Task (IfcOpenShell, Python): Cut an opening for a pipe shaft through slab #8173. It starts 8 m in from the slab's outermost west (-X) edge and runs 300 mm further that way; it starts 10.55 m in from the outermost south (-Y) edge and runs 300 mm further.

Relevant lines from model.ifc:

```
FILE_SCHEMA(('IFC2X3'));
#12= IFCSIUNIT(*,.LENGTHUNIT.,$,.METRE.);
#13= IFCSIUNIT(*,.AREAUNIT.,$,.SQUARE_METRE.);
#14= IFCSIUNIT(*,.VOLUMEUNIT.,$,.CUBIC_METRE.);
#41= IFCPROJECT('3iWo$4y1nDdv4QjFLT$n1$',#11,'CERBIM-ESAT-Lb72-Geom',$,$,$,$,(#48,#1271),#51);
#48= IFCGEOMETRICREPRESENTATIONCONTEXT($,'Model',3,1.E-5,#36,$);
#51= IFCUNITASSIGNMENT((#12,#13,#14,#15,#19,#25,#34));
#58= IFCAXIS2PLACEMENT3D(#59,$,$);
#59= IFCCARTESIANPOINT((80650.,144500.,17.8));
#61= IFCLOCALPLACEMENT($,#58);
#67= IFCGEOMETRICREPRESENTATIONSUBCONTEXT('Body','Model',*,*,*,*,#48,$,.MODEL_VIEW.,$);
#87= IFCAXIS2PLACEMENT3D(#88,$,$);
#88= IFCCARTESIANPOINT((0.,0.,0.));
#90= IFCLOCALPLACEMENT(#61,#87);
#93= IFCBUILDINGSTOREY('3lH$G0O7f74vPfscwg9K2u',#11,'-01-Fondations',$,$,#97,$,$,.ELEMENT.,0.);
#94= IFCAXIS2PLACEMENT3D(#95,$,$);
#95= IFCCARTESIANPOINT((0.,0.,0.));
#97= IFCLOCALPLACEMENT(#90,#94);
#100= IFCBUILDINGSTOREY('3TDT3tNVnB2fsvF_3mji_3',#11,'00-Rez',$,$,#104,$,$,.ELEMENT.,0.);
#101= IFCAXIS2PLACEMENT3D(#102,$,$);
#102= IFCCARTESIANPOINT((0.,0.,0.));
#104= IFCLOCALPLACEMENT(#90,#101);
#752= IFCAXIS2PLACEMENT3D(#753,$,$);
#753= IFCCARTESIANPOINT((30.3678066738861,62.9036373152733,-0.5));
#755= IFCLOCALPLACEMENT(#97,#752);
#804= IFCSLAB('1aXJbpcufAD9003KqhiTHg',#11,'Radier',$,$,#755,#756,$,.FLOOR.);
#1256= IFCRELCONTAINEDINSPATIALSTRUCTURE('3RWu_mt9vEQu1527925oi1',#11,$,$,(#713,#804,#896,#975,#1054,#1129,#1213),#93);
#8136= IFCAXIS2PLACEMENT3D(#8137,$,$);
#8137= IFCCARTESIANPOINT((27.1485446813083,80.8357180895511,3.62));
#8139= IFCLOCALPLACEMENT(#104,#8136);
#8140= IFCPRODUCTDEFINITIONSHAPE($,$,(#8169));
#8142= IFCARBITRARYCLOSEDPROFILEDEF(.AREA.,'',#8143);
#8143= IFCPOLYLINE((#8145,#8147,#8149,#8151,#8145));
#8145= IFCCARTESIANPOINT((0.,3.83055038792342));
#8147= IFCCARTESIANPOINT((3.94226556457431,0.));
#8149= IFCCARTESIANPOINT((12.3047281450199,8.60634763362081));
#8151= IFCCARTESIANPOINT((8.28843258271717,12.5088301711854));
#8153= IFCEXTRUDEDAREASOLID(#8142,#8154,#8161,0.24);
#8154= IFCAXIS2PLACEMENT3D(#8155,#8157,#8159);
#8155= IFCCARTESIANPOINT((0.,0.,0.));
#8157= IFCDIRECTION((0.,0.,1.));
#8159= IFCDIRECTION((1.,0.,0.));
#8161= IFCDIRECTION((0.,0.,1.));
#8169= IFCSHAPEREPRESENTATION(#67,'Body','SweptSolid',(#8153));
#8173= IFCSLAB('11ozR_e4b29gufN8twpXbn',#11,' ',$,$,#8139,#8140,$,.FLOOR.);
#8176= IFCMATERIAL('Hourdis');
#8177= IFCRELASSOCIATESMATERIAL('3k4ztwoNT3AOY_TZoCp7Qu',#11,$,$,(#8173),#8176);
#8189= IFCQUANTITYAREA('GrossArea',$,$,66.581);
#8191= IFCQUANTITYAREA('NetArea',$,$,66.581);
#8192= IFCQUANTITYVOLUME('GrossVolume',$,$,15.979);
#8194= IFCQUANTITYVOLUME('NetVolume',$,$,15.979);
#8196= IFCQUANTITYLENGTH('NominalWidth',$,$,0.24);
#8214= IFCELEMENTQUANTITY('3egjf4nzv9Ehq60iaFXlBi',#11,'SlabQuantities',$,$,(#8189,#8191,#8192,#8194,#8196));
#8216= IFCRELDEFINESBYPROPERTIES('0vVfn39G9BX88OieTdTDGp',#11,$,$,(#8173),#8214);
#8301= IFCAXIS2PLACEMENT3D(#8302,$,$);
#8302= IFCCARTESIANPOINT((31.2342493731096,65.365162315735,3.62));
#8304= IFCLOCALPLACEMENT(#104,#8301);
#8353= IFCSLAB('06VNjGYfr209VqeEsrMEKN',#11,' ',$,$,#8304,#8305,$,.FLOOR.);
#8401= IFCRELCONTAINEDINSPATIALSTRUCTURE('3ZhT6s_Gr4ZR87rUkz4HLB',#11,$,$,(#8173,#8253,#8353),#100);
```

```python
import numpy as np
import ifcopenshell
import ifcopenshell.api.feature
import ifcopenshell.api.geometry
import ifcopenshell.api.pset
import ifcopenshell.api.root
import ifcopenshell.geom
import ifcopenshell.util.element
import ifcopenshell.util.placement
import ifcopenshell.util.representation
import ifcopenshell.util.shape
import ifcopenshell.util.unit

model = ifcopenshell.open("model.ifc")
unit_scale = ifcopenshell.util.unit.calculate_unit_scale(model)
area_scale = ifcopenshell.util.unit.calculate_unit_scale(model, "AREAUNIT")
volume_scale = ifcopenshell.util.unit.calculate_unit_scale(model, "VOLUMEUNIT")
settings = ifcopenshell.geom.settings()


def volume(element):
    """Net volume in cubic metres, openings subtracted."""
    shape = ifcopenshell.geom.create_shape(settings, element)
    return ifcopenshell.util.shape.get_volume(shape.geometry)


slab = model.by_id(8173)
before = volume(slab)

# Extent in the slab's own axes, in metres. The edges named are its -X and -Y sides.
slab_shape = ifcopenshell.geom.create_shape(settings, slab)
vertices = ifcopenshell.util.shape.get_vertices(slab_shape.geometry)
x_min, y_min, bottom = vertices.min(axis=0)
top = vertices[:, 2].max()

opening = ifcopenshell.api.root.create_entity(model, ifc_class="IfcOpeningElement", name="Pipe shaft opening")
context = ifcopenshell.util.representation.get_context(model, "Model", "Body", "MODEL_VIEW")
width, depth = 0.3, 0.3
outline = [(0.0, 0.0), (width, 0.0), (width, depth), (0.0, depth), (0.0, 0.0)]
# Overshoot both faces by 50 mm so the cut is clean.
shape = ifcopenshell.api.geometry.add_slab_representation(
    model, context=context, depth=top - bottom + 0.1, polyline=outline
)
ifcopenshell.api.geometry.assign_representation(model, product=opening, representation=shape)

matrix = ifcopenshell.util.placement.get_local_placement(slab.ObjectPlacement)
matrix[:, 3] = matrix @ np.append(np.array([x_min + 8, y_min + 10.55, bottom - 0.05]) / unit_scale, 1.0)
ifcopenshell.api.geometry.edit_object_placement(model, product=opening, matrix=matrix, is_si=False)
ifcopenshell.api.feature.add_feature(model, feature=opening, element=slab)

after = volume(slab)

# Update the slab's stored quantities.
qto = model.by_id(ifcopenshell.util.element.get_pset(slab, "SlabQuantities", should_inherit=False)["id"])
ifcopenshell.api.pset.edit_qto(model, qto=qto, properties={
    "NetArea": after / (top - bottom) / area_scale,
    "NetVolume": after / volume_scale,
})

print(f"slab volume {before:.3f} -> {after:.3f} m3")

model.write("model_rev.ifc")
```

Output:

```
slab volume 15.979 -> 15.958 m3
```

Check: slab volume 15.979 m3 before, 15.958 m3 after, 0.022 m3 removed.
